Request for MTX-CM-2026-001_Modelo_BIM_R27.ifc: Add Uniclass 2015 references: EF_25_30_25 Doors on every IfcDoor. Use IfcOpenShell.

First a look at what the model holds.

```python
import ifcopenshell

model = ifcopenshell.open("MTX-CM-2026-001_Modelo_BIM_R27.ifc")
print(model.schema)
print("classifications:", [c.Name for c in model.by_type("IfcClassification")])
for ifc_class in ("IfcDoor", "IfcRoof", "IfcStair", "IfcWall", "IfcWindow"):
    print(ifc_class, len(model.by_type(ifc_class)))
```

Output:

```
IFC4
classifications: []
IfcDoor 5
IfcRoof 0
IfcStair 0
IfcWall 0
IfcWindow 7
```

```python
import ifcopenshell
import ifcopenshell.api.classification

model = ifcopenshell.open("MTX-CM-2026-001_Modelo_BIM_R27.ifc")

system = ifcopenshell.api.classification.add_classification(model, classification="Uniclass 2015")

codes = {
    "IfcDoor": ("EF_25_30_25", "Doors"),
}
for ifc_class, (code, name) in codes.items():
    products = model.by_type(ifc_class)
    ifcopenshell.api.classification.add_reference(
        model, products=products, classification=system, identification=code, name=name
    )
    print(code, len(products))

model.write("MTX-CM-2026-001_Modelo_BIM_R27-out.ifc")
```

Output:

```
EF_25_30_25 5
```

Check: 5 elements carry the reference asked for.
